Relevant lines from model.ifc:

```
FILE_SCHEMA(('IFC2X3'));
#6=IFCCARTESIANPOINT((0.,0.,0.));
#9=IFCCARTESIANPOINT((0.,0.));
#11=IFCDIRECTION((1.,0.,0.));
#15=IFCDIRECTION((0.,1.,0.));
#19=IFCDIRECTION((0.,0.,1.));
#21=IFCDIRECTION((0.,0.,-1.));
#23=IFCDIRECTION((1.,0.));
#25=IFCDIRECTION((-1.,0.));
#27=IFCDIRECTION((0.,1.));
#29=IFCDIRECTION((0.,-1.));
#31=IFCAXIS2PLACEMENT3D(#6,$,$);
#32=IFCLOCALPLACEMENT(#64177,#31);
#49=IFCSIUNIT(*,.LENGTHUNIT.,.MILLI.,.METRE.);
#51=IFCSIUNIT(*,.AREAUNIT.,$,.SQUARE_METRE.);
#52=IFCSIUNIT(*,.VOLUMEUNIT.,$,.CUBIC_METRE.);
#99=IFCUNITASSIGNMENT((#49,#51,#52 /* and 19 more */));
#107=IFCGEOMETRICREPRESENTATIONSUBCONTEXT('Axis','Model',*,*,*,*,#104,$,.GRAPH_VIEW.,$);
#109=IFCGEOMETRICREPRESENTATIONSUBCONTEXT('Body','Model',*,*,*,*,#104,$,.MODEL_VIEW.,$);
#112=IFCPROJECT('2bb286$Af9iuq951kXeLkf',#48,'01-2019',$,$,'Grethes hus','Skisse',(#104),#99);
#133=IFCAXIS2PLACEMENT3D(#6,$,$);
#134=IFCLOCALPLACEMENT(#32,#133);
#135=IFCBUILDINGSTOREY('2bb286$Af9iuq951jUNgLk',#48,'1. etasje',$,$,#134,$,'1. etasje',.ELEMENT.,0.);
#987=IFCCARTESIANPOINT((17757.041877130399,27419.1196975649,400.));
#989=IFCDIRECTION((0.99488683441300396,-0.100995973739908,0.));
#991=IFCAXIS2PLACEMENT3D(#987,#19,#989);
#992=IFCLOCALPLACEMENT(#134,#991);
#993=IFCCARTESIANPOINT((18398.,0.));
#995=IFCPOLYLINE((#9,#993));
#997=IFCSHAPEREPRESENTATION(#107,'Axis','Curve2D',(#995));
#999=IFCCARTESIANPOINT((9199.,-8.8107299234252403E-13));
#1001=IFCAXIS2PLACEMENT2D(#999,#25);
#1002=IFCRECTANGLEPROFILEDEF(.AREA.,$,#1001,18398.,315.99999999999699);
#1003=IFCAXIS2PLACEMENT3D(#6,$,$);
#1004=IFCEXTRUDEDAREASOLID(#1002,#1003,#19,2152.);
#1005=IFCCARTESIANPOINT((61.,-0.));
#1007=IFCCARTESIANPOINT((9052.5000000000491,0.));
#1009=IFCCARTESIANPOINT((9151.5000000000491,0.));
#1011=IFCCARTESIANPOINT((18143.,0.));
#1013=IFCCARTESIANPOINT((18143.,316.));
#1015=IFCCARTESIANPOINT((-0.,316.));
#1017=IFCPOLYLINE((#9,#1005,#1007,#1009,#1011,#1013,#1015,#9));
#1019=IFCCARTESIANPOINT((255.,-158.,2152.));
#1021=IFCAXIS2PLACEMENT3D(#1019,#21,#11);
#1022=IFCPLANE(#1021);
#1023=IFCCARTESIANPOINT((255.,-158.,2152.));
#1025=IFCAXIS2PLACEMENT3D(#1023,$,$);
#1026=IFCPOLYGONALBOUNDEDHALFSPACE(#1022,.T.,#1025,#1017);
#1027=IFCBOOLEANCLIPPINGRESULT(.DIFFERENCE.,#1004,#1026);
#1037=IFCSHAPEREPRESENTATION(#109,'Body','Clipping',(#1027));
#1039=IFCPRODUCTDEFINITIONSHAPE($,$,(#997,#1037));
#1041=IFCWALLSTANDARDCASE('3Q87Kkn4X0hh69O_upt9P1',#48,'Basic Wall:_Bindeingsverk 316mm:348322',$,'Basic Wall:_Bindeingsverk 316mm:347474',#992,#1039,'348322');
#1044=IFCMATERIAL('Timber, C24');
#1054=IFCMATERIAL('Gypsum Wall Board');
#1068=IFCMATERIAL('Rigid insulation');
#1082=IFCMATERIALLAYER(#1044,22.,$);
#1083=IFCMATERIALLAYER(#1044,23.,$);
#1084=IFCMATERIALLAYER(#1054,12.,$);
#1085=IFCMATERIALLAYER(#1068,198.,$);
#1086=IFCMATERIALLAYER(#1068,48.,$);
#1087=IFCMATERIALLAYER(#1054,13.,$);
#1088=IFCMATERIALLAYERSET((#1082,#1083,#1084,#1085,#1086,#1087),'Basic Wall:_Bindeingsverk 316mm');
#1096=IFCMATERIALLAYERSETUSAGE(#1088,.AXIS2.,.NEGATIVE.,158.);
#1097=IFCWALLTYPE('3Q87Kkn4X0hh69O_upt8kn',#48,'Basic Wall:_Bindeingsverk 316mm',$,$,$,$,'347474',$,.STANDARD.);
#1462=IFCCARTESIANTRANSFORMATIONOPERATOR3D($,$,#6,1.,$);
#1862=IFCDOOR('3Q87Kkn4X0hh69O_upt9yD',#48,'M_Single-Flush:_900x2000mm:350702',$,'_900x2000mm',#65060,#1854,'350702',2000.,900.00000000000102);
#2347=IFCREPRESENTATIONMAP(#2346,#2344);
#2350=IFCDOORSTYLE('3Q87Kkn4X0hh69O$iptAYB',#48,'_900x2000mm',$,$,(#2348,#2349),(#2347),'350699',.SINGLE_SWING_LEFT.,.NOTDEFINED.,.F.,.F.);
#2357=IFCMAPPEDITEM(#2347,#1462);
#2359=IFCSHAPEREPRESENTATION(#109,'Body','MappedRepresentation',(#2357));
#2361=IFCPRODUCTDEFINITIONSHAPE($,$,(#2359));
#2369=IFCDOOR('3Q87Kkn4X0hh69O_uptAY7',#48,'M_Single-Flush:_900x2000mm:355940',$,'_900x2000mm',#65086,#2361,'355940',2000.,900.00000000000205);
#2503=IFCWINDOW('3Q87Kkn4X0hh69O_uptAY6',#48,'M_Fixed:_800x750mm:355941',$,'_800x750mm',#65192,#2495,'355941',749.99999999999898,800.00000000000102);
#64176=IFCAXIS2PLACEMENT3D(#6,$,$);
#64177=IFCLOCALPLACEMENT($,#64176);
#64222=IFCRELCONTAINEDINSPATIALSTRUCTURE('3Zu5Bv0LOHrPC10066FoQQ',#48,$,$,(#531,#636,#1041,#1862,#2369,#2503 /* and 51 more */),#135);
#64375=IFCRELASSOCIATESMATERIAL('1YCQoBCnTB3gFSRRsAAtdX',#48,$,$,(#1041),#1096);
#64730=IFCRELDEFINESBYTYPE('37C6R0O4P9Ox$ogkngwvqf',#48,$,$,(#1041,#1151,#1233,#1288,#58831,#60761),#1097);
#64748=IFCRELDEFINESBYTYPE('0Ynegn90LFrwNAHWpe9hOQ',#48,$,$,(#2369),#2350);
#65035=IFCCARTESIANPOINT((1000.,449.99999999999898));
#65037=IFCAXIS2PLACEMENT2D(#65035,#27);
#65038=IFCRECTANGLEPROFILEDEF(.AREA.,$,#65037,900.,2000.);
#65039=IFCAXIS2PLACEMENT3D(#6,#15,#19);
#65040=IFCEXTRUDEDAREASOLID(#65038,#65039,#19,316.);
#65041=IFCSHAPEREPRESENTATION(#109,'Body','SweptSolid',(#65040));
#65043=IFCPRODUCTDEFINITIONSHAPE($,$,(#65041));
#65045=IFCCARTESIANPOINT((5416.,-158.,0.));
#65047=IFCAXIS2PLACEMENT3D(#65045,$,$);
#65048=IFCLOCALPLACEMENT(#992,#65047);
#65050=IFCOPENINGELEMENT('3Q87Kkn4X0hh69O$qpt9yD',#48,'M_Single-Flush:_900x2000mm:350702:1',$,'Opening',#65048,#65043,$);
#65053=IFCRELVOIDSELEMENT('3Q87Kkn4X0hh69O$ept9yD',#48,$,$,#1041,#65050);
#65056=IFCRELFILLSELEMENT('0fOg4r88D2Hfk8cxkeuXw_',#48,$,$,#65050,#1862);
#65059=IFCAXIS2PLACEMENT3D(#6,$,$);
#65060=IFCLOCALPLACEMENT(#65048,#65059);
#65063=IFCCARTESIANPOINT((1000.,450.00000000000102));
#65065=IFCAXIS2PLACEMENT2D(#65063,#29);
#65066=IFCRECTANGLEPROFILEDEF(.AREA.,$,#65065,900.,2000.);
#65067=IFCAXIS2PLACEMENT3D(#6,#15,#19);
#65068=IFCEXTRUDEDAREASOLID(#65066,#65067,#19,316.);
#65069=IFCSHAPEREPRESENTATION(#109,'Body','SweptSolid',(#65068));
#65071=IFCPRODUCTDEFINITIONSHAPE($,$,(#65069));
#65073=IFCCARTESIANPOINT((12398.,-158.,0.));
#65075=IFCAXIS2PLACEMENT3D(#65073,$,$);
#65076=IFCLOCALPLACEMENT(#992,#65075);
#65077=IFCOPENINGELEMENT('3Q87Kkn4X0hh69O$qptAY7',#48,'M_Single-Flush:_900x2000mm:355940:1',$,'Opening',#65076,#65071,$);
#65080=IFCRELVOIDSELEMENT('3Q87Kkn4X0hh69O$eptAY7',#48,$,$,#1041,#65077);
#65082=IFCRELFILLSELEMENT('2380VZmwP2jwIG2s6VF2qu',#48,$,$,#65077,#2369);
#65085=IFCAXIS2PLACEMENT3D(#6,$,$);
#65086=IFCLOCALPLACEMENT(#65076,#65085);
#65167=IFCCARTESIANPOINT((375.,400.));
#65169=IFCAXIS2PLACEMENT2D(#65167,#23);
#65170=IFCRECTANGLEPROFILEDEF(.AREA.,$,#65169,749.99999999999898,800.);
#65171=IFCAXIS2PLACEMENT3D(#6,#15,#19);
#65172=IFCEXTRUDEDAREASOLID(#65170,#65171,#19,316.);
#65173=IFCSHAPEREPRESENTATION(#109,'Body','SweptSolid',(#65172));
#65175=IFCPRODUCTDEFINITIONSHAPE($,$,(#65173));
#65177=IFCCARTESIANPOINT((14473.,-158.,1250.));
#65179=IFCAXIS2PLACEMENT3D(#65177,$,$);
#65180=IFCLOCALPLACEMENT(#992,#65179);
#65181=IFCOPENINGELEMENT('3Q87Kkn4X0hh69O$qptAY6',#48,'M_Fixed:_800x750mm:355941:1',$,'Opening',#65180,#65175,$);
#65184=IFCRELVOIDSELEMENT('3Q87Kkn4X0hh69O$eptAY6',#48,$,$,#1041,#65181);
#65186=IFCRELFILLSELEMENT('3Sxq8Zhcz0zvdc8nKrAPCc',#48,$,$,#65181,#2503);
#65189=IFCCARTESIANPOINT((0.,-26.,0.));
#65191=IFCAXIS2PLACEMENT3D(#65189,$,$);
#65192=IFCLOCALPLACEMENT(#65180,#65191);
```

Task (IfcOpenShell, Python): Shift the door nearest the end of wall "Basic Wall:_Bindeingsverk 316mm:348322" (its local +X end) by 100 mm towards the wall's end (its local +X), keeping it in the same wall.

```python
import ifcopenshell
import ifcopenshell.api.geometry
import ifcopenshell.util.placement

model = ifcopenshell.open("model.ifc")

door = model.by_id(2369)
opening = door.FillsVoids[0].RelatingOpeningElement
wall = opening.VoidsElements[0].RelatingBuildingElement

wall_matrix = ifcopenshell.util.placement.get_local_placement(wall.ObjectPlacement)
shift = wall_matrix[:3, 0] * 100.0
before = ifcopenshell.util.placement.get_local_placement(door.ObjectPlacement)[:3, 3].copy()

# The door is placed relative to its opening, so it follows when the opening moves.
matrix = ifcopenshell.util.placement.get_local_placement(opening.ObjectPlacement)
matrix[:3, 3] += shift
ifcopenshell.api.geometry.edit_object_placement(
    model, product=opening, matrix=matrix, is_si=False, should_transform_children=True
)

after = ifcopenshell.util.placement.get_local_placement(door.ObjectPlacement)[:3, 3]
print("door moved by", (after - before).round(3) + 0.0)

model.write("model_rev.ifc")
```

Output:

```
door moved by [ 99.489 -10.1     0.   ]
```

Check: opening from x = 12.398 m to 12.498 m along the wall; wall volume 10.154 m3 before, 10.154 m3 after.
